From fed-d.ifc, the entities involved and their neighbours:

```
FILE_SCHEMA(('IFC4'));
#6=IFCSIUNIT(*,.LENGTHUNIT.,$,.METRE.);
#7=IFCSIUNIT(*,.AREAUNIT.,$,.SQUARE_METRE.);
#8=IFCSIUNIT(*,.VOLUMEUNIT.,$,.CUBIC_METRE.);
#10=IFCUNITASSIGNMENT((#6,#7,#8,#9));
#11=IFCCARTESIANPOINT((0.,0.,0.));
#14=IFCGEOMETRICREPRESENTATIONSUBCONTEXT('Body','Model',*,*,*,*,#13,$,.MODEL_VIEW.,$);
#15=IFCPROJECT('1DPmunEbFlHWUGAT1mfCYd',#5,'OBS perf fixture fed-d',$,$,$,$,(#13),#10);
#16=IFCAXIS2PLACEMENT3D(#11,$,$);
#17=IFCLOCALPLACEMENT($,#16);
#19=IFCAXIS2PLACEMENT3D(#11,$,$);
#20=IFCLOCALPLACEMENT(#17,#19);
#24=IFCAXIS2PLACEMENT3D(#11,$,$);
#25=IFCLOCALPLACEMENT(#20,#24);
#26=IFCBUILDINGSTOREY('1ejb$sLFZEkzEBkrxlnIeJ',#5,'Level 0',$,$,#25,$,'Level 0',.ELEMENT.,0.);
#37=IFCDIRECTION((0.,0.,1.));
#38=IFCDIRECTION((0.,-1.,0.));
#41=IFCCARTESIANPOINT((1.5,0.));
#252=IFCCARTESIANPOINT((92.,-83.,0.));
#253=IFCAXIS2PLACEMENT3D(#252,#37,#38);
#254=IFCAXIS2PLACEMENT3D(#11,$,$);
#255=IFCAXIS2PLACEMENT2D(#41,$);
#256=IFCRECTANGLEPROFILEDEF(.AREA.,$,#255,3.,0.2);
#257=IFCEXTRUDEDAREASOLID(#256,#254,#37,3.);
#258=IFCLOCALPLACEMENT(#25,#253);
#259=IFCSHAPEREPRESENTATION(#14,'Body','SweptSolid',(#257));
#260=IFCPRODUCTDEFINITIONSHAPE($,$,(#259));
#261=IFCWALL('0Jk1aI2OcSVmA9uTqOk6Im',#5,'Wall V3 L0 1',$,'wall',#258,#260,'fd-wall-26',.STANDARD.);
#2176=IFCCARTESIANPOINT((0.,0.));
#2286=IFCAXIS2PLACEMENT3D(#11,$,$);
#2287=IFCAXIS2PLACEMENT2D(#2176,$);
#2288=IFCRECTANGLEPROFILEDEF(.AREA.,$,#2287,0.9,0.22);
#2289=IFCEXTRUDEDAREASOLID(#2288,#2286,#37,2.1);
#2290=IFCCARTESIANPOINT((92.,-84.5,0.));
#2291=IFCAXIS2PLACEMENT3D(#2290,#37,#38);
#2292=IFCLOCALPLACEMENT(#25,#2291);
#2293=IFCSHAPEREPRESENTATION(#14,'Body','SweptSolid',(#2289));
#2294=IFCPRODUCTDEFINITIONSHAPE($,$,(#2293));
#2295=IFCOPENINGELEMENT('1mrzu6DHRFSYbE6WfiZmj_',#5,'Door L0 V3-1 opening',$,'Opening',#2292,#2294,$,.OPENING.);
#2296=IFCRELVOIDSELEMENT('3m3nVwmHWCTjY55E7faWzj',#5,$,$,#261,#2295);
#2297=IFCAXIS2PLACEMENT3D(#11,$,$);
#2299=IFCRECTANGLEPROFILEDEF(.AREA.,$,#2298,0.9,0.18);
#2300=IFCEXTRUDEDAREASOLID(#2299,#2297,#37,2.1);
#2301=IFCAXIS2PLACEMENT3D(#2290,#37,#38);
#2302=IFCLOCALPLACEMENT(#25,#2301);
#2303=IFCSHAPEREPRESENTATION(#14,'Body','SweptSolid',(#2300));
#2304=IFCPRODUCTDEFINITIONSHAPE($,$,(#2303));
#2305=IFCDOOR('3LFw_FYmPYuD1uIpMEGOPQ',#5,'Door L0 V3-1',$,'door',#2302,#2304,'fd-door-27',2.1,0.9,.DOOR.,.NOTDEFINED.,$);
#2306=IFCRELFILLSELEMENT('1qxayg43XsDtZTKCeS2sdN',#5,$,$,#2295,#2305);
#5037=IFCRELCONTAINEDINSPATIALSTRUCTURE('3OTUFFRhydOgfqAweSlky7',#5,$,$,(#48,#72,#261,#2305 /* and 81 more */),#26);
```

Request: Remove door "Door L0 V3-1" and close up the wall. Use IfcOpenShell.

```python
import ifcopenshell
import ifcopenshell.api.feature
import ifcopenshell.api.root
import ifcopenshell.geom
import ifcopenshell.util.shape

model = ifcopenshell.open("fed-d.ifc")
settings = ifcopenshell.geom.settings()


def volume(element):
    """Net volume in cubic metres, openings subtracted."""
    shape = ifcopenshell.geom.create_shape(settings, element)
    return ifcopenshell.util.shape.get_volume(shape.geometry)


door = model.by_guid("3LFw_FYmPYuD1uIpMEGOPQ")
opening = door.FillsVoids[0].RelatingOpeningElement
wall = opening.VoidsElements[0].RelatingBuildingElement
before = volume(wall)

ifcopenshell.api.root.remove_product(model, product=door)
ifcopenshell.api.feature.remove_feature(model, feature=opening)

after = volume(wall)

print(f"wall volume {before:.3f} -> {after:.3f} m3")

model.write("fed-d_updated.ifc")
```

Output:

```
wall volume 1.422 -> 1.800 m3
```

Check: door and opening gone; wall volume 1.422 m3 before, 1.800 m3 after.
